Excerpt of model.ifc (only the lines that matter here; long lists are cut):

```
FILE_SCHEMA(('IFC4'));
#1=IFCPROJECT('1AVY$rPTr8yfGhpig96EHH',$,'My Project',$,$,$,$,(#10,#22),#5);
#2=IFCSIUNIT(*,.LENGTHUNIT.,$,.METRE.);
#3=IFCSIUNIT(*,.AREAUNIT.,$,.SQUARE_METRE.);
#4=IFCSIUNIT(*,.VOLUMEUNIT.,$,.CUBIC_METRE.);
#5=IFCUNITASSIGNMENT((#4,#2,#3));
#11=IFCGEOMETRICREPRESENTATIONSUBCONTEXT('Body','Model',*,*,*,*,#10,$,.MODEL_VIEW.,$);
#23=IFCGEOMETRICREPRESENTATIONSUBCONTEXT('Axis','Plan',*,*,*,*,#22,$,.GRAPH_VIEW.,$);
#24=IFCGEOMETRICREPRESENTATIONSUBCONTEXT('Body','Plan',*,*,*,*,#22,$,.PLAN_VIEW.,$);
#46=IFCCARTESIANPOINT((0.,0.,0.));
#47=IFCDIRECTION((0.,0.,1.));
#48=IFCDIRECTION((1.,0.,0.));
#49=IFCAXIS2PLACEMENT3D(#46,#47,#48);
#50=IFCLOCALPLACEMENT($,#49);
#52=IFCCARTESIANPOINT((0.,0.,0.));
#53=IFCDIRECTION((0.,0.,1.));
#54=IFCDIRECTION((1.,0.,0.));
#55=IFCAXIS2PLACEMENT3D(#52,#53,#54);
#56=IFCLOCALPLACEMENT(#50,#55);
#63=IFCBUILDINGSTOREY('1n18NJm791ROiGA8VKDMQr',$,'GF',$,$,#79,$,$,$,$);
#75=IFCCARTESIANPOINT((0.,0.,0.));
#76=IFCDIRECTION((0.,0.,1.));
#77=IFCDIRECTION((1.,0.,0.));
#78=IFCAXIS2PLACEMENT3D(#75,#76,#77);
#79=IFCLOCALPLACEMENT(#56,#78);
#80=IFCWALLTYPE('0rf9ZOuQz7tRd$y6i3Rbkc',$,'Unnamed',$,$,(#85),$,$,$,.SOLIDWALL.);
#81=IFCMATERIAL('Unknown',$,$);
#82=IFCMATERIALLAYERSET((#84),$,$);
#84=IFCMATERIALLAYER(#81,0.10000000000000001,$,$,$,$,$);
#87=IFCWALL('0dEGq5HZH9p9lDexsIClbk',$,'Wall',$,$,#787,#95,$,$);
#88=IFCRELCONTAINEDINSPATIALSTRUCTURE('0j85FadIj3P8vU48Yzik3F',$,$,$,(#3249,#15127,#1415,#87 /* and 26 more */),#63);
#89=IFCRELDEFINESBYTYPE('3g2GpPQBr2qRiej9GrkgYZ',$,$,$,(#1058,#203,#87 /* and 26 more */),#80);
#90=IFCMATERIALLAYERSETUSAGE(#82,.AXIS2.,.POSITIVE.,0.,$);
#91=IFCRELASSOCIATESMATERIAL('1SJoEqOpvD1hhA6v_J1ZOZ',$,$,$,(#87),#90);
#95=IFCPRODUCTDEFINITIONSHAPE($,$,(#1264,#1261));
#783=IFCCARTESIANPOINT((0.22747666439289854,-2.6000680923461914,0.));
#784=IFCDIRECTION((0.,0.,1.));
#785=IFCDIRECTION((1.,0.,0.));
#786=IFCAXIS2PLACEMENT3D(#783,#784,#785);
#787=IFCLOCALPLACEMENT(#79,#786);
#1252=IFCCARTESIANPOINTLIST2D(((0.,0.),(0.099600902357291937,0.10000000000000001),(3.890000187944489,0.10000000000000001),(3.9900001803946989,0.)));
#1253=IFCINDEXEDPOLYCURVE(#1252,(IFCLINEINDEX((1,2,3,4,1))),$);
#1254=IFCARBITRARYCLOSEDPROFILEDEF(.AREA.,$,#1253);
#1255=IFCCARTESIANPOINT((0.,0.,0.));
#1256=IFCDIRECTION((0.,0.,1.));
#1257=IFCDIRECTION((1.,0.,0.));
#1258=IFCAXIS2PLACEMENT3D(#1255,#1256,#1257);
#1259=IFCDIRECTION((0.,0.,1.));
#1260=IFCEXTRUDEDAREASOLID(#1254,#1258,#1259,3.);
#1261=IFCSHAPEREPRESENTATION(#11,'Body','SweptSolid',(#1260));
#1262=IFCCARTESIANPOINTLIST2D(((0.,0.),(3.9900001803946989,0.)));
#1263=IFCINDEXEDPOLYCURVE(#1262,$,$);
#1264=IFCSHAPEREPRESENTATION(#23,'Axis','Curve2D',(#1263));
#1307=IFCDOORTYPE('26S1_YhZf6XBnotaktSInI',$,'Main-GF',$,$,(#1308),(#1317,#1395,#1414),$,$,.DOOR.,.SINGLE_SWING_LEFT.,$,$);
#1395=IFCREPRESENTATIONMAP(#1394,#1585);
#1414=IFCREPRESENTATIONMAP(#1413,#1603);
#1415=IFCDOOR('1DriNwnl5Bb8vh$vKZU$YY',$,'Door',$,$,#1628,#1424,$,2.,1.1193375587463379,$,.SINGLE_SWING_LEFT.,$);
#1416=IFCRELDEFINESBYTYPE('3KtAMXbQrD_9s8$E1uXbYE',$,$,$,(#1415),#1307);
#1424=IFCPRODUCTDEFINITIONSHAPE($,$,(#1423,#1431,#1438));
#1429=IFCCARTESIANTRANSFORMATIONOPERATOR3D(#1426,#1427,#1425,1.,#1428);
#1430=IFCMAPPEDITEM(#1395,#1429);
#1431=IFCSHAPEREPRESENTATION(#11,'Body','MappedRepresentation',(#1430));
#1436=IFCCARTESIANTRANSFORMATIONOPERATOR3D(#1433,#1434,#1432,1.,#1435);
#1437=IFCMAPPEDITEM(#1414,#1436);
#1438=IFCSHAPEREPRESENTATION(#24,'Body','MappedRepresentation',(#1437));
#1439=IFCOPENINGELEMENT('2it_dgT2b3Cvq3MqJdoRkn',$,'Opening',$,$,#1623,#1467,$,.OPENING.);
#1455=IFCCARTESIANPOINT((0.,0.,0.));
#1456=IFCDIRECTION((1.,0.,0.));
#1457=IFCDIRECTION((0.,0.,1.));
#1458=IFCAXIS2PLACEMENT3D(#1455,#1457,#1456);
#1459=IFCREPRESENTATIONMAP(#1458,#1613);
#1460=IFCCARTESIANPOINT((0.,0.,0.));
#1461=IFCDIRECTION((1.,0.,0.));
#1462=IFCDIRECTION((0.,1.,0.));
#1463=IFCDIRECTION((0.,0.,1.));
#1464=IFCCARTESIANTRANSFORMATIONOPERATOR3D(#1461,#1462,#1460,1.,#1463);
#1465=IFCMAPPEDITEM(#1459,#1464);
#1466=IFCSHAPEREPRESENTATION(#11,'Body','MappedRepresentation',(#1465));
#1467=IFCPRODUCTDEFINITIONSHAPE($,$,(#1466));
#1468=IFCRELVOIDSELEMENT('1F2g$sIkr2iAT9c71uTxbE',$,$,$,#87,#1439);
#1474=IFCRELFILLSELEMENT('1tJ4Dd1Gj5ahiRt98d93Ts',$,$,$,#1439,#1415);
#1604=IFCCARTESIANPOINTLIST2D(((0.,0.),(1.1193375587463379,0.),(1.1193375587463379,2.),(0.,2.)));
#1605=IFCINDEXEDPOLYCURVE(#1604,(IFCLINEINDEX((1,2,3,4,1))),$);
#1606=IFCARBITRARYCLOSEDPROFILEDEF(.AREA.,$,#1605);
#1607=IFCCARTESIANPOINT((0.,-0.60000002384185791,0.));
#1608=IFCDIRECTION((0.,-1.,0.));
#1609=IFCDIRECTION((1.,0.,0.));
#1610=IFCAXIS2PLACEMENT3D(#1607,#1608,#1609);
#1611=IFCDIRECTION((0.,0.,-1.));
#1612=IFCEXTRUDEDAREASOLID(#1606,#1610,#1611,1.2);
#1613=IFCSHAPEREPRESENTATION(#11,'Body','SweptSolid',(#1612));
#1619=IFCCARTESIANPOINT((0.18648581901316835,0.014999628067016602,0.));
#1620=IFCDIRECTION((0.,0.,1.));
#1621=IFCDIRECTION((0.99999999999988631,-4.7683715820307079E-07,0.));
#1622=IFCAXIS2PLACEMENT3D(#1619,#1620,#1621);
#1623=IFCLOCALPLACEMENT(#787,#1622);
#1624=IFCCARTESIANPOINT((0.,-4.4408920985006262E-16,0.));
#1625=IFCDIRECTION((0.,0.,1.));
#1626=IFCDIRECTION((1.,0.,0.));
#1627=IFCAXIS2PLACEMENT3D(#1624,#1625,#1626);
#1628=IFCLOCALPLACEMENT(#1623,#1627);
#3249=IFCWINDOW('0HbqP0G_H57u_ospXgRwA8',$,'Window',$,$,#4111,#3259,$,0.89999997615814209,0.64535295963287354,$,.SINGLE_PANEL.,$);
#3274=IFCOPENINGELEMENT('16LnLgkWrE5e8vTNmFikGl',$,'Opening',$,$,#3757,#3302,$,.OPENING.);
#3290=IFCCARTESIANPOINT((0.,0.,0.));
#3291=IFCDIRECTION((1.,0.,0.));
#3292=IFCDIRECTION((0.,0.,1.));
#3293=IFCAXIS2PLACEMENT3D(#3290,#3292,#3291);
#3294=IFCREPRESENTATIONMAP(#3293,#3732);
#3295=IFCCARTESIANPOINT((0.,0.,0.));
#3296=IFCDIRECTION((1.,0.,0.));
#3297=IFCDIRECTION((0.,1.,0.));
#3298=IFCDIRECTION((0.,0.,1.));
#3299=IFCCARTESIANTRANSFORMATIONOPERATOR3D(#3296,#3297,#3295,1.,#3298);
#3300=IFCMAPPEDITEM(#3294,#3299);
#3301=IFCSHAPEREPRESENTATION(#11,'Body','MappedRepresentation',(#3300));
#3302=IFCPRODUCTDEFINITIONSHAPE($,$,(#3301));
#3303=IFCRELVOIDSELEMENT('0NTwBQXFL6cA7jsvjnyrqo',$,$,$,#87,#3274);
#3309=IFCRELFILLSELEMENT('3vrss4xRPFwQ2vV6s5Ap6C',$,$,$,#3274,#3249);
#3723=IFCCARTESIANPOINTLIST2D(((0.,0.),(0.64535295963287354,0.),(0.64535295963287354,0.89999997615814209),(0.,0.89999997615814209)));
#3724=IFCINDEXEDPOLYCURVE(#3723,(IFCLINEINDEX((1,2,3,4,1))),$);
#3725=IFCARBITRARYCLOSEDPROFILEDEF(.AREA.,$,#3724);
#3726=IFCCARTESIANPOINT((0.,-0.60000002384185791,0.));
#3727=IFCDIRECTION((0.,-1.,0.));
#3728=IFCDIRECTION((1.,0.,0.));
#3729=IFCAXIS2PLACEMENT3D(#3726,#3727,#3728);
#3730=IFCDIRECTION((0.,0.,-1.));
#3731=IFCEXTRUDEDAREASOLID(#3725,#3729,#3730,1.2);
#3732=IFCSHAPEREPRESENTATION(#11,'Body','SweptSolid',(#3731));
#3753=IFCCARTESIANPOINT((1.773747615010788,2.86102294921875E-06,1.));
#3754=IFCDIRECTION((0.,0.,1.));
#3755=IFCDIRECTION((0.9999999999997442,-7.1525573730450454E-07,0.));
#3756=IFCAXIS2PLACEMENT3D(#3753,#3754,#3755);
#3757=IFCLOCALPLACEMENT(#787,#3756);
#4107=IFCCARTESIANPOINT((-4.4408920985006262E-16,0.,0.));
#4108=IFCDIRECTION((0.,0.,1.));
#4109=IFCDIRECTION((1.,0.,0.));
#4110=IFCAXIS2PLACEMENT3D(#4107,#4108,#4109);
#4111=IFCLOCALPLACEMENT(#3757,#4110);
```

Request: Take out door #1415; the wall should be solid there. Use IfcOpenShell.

```python
import ifcopenshell
import ifcopenshell.api.feature
import ifcopenshell.api.root
import ifcopenshell.geom
import ifcopenshell.util.shape

model = ifcopenshell.open("model.ifc")
settings = ifcopenshell.geom.settings()


def volume(element):
    """Net volume in cubic metres, openings subtracted."""
    shape = ifcopenshell.geom.create_shape(settings, element)
    return ifcopenshell.util.shape.get_volume(shape.geometry)


door = model.by_guid("1DriNwnl5Bb8vh$vKZU$YY")
opening = door.FillsVoids[0].RelatingOpeningElement
wall = opening.VoidsElements[0].RelatingBuildingElement
before = volume(wall)

ifcopenshell.api.root.remove_product(model, product=door)
ifcopenshell.api.feature.remove_feature(model, feature=opening)

after = volume(wall)

print(f"wall volume {before:.3f} -> {after:.3f} m3")

model.write("model-out.ifc")
```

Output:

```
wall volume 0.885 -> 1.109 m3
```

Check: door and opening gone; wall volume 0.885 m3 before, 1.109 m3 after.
